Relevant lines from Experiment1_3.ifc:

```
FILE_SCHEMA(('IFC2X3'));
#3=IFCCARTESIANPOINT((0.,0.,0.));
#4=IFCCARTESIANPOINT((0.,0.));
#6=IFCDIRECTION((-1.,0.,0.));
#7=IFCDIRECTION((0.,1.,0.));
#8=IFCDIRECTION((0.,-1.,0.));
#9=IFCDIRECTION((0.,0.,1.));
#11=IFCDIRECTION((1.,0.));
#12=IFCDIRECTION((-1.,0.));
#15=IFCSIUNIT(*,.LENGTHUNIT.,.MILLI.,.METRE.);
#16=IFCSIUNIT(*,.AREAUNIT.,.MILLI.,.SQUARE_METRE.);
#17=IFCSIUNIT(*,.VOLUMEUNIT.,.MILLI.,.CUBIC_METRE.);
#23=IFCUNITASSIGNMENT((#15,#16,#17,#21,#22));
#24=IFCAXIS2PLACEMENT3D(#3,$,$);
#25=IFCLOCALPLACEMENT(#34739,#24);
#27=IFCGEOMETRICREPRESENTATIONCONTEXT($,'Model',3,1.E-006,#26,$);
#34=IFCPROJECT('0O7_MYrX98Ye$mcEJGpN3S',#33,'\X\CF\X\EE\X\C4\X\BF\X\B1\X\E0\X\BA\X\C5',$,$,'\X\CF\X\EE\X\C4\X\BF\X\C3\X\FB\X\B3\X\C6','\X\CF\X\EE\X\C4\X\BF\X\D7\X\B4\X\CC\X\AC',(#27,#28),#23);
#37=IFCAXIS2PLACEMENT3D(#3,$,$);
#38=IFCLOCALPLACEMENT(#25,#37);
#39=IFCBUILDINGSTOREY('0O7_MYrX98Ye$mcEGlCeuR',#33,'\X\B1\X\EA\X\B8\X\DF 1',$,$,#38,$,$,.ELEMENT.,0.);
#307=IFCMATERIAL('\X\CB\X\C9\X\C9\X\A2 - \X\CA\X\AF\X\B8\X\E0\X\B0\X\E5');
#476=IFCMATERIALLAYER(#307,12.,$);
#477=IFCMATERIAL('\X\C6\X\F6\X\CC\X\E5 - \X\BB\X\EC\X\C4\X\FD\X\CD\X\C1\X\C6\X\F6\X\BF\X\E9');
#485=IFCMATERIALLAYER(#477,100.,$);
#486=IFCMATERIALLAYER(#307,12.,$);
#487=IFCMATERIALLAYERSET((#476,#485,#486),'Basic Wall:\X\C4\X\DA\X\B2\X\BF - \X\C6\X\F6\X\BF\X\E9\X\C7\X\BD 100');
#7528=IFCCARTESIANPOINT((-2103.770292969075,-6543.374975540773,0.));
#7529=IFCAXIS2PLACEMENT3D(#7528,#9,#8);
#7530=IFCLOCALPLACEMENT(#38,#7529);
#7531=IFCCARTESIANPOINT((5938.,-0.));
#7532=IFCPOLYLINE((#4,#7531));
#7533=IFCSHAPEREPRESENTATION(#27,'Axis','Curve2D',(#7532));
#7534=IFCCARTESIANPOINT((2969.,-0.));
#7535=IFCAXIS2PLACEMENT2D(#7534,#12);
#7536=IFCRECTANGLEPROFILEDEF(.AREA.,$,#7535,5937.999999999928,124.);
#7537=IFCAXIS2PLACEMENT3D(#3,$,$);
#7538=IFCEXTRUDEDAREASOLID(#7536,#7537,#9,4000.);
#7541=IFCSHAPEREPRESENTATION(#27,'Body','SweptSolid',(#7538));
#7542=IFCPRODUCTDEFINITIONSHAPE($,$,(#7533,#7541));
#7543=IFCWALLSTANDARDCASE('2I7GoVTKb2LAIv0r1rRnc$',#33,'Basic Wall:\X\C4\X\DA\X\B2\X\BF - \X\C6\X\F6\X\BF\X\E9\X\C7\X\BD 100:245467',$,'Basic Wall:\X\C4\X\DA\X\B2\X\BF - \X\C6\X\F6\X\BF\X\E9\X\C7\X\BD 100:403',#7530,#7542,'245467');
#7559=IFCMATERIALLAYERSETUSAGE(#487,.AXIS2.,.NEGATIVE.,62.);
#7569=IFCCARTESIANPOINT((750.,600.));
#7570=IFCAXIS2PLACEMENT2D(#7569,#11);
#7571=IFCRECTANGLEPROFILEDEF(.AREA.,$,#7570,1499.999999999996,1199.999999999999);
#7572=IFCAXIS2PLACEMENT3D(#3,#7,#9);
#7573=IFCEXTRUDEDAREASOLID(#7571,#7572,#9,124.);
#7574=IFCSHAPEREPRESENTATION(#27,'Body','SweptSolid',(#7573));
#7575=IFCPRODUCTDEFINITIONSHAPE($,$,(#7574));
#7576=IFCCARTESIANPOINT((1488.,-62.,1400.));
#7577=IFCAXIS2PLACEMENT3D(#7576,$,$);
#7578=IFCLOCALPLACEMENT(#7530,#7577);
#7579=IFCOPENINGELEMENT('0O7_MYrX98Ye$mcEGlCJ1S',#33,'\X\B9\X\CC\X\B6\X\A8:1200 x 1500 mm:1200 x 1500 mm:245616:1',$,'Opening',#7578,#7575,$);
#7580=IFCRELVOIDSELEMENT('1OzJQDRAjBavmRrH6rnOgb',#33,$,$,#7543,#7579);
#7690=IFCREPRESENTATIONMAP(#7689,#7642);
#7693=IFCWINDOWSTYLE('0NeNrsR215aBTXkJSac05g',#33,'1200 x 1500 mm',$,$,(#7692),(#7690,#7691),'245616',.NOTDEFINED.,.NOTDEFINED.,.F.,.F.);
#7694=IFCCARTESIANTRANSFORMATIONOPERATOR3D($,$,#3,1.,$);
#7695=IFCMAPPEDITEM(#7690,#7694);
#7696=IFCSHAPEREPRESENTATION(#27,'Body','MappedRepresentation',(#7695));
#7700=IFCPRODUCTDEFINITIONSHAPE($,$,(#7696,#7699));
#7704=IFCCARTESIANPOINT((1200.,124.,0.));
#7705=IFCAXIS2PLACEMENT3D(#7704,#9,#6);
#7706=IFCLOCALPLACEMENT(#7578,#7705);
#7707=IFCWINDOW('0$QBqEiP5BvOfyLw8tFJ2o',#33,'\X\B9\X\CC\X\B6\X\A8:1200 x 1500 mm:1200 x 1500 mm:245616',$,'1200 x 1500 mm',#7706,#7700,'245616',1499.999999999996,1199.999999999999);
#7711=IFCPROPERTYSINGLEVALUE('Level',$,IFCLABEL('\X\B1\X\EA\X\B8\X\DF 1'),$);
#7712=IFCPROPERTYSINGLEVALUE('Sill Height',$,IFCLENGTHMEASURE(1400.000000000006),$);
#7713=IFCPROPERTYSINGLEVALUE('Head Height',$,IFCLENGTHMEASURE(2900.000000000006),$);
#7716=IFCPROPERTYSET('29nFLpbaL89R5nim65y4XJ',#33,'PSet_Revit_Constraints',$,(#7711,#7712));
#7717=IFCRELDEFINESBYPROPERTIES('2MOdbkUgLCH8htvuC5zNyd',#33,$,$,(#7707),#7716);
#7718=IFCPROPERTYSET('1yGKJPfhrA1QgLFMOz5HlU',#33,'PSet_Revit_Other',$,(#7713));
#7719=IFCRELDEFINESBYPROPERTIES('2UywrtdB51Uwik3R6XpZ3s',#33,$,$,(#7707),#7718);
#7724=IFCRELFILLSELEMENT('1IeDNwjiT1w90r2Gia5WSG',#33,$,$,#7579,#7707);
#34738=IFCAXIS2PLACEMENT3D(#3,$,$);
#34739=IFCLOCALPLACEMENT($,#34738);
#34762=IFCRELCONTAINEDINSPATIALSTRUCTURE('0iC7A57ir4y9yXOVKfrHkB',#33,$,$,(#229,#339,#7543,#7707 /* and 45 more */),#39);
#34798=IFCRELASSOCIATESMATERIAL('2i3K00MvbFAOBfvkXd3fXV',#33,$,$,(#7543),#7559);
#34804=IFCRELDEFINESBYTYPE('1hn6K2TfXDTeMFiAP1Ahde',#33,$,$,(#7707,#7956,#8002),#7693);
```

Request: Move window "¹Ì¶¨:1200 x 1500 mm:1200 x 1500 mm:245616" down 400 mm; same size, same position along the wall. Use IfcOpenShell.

```python
import numpy as np
import ifcopenshell
import ifcopenshell.api.geometry
import ifcopenshell.api.pset
import ifcopenshell.util.element
import ifcopenshell.util.placement
import ifcopenshell.util.unit

model = ifcopenshell.open("Experiment1_3.ifc")
unit_scale = ifcopenshell.util.unit.calculate_unit_scale(model)

window = model.by_guid("0$QBqEiP5BvOfyLw8tFJ2o")
opening = window.FillsVoids[0].RelatingOpeningElement
dz = -400.0

shift = np.array([0.0, 0.0, dz])
# The window is placed relative to its opening, so it follows when the opening moves.
matrix = ifcopenshell.util.placement.get_local_placement(opening.ObjectPlacement)
matrix[:3, 3] += shift
ifcopenshell.api.geometry.edit_object_placement(
    model, product=opening, matrix=matrix, is_si=False, should_transform_children=True
)

# Keep the stored heights in step.
pset = model.by_id(ifcopenshell.util.element.get_pset(window, "PSet_Revit_Constraints", should_inherit=False)["id"])
ifcopenshell.api.pset.edit_pset(model, pset=pset, properties={
    "Sill Height": model.create_entity("IfcLengthMeasure", ifcopenshell.util.element.get_pset(window, "PSet_Revit_Constraints", "Sill Height") + dz),
})
pset = model.by_id(ifcopenshell.util.element.get_pset(window, "PSet_Revit_Other", should_inherit=False)["id"])
ifcopenshell.api.pset.edit_pset(model, pset=pset, properties={
    "Head Height": model.create_entity("IfcLengthMeasure", ifcopenshell.util.element.get_pset(window, "PSet_Revit_Other", "Head Height") + dz),
})

print(f"moved by {dz * unit_scale:+.3f} m")

model.write("Experiment1_3_rev.ifc")
```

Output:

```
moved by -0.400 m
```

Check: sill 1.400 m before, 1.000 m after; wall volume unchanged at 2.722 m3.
